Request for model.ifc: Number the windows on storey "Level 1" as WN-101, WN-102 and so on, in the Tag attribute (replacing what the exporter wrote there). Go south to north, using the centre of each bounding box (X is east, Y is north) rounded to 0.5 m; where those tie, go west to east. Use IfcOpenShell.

First a look at what the model holds.

```python
import ifcopenshell
import ifcopenshell.util.element
import ifcopenshell.util.placement

model = ifcopenshell.open("model.ifc")
print(model.schema)
storey = next(s for s in model.by_type("IfcBuildingStorey") if s.Name == "Level 1")
windows = [e for e in ifcopenshell.util.element.get_decomposition(storey) if e.is_a("IfcWindow")]
for e in sorted(windows, key=lambda e: e.id()):
    origin = ifcopenshell.util.placement.get_local_placement(e.ObjectPlacement)[:3, 3]
    print(e.id(), e.Tag, e.Name, origin.round(2) + 0.0, sep=" | ")
```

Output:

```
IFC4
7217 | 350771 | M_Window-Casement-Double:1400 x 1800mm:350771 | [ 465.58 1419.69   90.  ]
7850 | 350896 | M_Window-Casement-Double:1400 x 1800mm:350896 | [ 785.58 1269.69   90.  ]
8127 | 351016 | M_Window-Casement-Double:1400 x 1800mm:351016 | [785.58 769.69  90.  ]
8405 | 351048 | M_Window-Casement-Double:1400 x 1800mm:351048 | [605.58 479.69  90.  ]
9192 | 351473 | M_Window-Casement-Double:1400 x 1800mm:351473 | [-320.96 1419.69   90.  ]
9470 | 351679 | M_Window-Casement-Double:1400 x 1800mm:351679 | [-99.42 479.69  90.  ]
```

```python
import ifcopenshell
import ifcopenshell.geom
import ifcopenshell.util.element
import ifcopenshell.util.shape

model = ifcopenshell.open("model.ifc")
settings = ifcopenshell.geom.settings()
settings.set("use-world-coords", True)


def centre(element):
    shape = ifcopenshell.geom.create_shape(settings, element)
    return ifcopenshell.util.shape.get_bbox_centroid(shape.geometry)


storey = next(s for s in model.by_type("IfcBuildingStorey") if s.Name == "Level 1")
windows = [e for e in ifcopenshell.util.element.get_decomposition(storey) if e.is_a("IfcWindow")]

# Insertion points can sit at a corner or the storey origin, so sort by the geometry (in metres).
centres = {e: centre(e) for e in windows}
windows.sort(key=lambda e: (round(centres[e][1] / 0.5), centres[e][0]))

for i, e in enumerate(windows, start=1):
    number = f"WN-1{i:02d}"
    e.Tag = number
    print(e.id(), number)

model.write("model_v2.ifc")
```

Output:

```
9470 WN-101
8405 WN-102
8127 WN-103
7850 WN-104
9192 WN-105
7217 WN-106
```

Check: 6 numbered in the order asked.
